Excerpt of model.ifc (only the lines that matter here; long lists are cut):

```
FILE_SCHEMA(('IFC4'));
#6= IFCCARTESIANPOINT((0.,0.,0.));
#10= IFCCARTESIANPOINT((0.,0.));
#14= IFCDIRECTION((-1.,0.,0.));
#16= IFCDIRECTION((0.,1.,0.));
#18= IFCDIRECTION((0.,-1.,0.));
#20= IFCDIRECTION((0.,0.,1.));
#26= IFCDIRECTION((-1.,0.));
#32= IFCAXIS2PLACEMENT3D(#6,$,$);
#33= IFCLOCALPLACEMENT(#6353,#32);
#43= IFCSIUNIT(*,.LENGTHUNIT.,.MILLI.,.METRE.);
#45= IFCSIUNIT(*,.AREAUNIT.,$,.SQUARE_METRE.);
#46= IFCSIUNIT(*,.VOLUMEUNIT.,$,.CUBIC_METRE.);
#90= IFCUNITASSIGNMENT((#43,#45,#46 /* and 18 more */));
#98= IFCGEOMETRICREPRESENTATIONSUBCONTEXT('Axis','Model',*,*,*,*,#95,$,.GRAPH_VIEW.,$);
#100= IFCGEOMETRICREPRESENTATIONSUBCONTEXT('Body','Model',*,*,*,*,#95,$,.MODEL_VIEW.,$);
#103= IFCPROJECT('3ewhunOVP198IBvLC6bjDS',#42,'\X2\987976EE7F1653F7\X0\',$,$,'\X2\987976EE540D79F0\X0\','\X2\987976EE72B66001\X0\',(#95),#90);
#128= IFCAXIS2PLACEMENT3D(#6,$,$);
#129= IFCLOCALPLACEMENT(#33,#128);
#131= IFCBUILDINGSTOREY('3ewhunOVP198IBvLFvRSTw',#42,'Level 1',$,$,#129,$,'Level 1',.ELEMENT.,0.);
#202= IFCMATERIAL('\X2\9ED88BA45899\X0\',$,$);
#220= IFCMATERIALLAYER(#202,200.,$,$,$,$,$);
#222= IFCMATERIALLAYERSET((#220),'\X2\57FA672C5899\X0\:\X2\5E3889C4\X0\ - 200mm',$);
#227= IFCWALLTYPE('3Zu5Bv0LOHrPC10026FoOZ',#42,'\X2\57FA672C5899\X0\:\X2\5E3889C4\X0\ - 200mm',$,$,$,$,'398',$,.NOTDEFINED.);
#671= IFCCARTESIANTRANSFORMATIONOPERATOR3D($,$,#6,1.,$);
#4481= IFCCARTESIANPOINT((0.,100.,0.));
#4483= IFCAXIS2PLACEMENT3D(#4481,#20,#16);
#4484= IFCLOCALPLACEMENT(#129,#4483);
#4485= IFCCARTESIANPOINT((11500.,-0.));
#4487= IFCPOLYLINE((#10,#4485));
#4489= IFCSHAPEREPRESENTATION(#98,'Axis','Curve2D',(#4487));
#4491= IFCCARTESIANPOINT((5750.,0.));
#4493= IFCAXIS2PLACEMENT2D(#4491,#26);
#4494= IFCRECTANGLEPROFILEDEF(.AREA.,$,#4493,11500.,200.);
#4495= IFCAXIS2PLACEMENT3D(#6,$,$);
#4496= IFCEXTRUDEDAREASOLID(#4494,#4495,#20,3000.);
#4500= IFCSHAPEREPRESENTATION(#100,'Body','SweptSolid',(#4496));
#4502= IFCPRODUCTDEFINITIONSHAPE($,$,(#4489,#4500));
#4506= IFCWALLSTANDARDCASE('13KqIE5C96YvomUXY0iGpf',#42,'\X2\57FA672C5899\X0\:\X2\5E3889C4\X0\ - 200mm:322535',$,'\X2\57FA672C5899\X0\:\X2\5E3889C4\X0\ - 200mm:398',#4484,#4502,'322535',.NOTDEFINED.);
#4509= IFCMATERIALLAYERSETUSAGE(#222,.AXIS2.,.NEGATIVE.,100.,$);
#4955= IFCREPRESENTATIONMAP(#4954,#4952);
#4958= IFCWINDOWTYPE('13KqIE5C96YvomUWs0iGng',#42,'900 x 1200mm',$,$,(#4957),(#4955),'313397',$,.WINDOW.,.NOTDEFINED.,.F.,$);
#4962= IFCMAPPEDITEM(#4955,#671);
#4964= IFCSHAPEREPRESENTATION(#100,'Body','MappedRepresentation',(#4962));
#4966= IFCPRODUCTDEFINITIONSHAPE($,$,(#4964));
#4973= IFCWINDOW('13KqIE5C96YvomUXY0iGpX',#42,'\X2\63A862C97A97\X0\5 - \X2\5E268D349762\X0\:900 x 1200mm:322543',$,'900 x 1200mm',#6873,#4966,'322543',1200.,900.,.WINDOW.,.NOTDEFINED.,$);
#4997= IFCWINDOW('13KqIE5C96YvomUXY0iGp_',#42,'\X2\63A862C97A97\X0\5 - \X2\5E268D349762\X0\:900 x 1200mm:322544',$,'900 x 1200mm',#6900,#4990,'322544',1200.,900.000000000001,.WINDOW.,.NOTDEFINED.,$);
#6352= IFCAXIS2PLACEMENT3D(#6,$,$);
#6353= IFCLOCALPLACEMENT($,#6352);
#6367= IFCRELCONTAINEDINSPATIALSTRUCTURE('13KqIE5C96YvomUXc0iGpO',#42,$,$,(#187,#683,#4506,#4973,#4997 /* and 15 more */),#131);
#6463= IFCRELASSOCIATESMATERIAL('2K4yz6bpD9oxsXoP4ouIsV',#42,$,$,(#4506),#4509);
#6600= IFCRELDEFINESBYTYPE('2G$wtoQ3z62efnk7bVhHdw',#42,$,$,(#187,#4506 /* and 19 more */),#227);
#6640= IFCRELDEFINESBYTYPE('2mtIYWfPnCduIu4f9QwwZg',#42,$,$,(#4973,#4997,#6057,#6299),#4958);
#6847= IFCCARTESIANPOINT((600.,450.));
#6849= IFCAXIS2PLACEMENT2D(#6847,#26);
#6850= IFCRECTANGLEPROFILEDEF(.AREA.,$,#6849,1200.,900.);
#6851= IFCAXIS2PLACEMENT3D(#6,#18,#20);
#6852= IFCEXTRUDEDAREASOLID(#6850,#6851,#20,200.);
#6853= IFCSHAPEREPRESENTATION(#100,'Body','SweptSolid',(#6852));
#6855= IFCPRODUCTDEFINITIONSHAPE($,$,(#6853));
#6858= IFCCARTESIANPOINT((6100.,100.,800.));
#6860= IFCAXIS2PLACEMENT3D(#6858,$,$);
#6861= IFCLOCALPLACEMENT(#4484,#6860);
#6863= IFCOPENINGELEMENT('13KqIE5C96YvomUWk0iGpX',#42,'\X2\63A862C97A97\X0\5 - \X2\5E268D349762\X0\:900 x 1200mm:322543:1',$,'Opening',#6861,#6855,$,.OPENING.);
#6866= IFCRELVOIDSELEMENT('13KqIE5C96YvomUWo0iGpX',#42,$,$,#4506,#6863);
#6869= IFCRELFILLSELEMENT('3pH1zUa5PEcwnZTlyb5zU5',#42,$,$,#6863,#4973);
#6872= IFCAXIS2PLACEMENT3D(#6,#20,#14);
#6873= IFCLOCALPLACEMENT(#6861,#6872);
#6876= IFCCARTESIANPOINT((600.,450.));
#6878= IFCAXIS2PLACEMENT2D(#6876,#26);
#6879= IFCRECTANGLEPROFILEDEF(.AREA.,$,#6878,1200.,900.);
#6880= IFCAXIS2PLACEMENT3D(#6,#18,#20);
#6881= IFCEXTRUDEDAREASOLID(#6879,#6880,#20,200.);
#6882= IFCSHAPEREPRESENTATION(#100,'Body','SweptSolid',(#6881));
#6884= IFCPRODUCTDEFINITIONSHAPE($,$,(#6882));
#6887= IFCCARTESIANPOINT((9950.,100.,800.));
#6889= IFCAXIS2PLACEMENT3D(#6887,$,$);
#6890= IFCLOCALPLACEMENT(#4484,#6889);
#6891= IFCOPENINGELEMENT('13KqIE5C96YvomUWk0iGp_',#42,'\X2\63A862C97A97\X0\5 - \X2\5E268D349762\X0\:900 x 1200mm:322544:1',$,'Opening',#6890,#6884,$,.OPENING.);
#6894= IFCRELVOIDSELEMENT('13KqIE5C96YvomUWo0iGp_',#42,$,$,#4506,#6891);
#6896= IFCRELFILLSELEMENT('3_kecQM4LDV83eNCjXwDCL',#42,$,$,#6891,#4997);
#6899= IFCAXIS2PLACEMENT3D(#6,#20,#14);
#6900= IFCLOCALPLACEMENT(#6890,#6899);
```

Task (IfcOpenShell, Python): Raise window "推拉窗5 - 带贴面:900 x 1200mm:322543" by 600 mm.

```python
import numpy as np
import ifcopenshell
import ifcopenshell.api.geometry
import ifcopenshell.util.placement
import ifcopenshell.util.unit

model = ifcopenshell.open("model.ifc")
unit_scale = ifcopenshell.util.unit.calculate_unit_scale(model)

window = model.by_guid("13KqIE5C96YvomUXY0iGpX")
opening = window.FillsVoids[0].RelatingOpeningElement
dz = 0.6 / unit_scale

shift = np.array([0.0, 0.0, dz])
# The window is placed relative to its opening, so it follows when the opening moves.
matrix = ifcopenshell.util.placement.get_local_placement(opening.ObjectPlacement)
matrix[:3, 3] += shift
ifcopenshell.api.geometry.edit_object_placement(
    model, product=opening, matrix=matrix, is_si=False, should_transform_children=True
)

print(f"moved by {dz * unit_scale:+.3f} m")

model.write("model-out.ifc")
```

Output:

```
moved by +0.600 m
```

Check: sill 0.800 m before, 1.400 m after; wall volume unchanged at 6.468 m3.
